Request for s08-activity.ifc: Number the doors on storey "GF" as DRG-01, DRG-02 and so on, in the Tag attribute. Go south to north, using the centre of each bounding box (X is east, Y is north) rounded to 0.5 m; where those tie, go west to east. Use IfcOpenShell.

First a look at what the model holds.

```python
import ifcopenshell
import ifcopenshell.util.element
import ifcopenshell.util.placement

model = ifcopenshell.open("s08-activity.ifc")
print(model.schema)
storey = next(s for s in model.by_type("IfcBuildingStorey") if s.Name == "GF")
doors = [e for e in ifcopenshell.util.element.get_decomposition(storey) if e.is_a("IfcDoor")]
for e in sorted(doors, key=lambda e: e.id()):
    origin = ifcopenshell.util.placement.get_local_placement(e.ObjectPlacement)[:3, 3]
    print(e.id(), e.Tag, e.Name, origin.round(2) + 0.0, sep=" | ")
```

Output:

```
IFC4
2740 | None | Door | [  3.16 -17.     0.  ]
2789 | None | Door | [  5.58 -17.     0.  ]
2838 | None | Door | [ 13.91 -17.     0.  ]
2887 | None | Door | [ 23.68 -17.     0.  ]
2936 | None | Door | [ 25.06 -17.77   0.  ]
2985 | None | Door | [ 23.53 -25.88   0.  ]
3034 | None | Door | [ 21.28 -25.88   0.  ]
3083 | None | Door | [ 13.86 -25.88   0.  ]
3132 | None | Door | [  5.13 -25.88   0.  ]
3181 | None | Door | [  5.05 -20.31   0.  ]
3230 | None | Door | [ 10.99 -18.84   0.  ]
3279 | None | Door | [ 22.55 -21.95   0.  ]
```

```python
import ifcopenshell
import ifcopenshell.geom
import ifcopenshell.util.element
import ifcopenshell.util.shape

model = ifcopenshell.open("s08-activity.ifc")
settings = ifcopenshell.geom.settings()
settings.set("use-world-coords", True)


def centre(element):
    shape = ifcopenshell.geom.create_shape(settings, element)
    return ifcopenshell.util.shape.get_bbox_centroid(shape.geometry)


storey = next(s for s in model.by_type("IfcBuildingStorey") if s.Name == "GF")
doors = [e for e in ifcopenshell.util.element.get_decomposition(storey) if e.is_a("IfcDoor")]

# Insertion points can sit at a corner or the storey origin, so sort by the geometry (in metres).
centres = {e: centre(e) for e in doors}
doors.sort(key=lambda e: (round(centres[e][1] / 0.5), centres[e][0]))

for i, e in enumerate(doors, start=1):
    number = f"DRG-{i:02d}"
    e.Tag = number
    print(e.id(), number)

model.write("s08-activity-out.ifc")
```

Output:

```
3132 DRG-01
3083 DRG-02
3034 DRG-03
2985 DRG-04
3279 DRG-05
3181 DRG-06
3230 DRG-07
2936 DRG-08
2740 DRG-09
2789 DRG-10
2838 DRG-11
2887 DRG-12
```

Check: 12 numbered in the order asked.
